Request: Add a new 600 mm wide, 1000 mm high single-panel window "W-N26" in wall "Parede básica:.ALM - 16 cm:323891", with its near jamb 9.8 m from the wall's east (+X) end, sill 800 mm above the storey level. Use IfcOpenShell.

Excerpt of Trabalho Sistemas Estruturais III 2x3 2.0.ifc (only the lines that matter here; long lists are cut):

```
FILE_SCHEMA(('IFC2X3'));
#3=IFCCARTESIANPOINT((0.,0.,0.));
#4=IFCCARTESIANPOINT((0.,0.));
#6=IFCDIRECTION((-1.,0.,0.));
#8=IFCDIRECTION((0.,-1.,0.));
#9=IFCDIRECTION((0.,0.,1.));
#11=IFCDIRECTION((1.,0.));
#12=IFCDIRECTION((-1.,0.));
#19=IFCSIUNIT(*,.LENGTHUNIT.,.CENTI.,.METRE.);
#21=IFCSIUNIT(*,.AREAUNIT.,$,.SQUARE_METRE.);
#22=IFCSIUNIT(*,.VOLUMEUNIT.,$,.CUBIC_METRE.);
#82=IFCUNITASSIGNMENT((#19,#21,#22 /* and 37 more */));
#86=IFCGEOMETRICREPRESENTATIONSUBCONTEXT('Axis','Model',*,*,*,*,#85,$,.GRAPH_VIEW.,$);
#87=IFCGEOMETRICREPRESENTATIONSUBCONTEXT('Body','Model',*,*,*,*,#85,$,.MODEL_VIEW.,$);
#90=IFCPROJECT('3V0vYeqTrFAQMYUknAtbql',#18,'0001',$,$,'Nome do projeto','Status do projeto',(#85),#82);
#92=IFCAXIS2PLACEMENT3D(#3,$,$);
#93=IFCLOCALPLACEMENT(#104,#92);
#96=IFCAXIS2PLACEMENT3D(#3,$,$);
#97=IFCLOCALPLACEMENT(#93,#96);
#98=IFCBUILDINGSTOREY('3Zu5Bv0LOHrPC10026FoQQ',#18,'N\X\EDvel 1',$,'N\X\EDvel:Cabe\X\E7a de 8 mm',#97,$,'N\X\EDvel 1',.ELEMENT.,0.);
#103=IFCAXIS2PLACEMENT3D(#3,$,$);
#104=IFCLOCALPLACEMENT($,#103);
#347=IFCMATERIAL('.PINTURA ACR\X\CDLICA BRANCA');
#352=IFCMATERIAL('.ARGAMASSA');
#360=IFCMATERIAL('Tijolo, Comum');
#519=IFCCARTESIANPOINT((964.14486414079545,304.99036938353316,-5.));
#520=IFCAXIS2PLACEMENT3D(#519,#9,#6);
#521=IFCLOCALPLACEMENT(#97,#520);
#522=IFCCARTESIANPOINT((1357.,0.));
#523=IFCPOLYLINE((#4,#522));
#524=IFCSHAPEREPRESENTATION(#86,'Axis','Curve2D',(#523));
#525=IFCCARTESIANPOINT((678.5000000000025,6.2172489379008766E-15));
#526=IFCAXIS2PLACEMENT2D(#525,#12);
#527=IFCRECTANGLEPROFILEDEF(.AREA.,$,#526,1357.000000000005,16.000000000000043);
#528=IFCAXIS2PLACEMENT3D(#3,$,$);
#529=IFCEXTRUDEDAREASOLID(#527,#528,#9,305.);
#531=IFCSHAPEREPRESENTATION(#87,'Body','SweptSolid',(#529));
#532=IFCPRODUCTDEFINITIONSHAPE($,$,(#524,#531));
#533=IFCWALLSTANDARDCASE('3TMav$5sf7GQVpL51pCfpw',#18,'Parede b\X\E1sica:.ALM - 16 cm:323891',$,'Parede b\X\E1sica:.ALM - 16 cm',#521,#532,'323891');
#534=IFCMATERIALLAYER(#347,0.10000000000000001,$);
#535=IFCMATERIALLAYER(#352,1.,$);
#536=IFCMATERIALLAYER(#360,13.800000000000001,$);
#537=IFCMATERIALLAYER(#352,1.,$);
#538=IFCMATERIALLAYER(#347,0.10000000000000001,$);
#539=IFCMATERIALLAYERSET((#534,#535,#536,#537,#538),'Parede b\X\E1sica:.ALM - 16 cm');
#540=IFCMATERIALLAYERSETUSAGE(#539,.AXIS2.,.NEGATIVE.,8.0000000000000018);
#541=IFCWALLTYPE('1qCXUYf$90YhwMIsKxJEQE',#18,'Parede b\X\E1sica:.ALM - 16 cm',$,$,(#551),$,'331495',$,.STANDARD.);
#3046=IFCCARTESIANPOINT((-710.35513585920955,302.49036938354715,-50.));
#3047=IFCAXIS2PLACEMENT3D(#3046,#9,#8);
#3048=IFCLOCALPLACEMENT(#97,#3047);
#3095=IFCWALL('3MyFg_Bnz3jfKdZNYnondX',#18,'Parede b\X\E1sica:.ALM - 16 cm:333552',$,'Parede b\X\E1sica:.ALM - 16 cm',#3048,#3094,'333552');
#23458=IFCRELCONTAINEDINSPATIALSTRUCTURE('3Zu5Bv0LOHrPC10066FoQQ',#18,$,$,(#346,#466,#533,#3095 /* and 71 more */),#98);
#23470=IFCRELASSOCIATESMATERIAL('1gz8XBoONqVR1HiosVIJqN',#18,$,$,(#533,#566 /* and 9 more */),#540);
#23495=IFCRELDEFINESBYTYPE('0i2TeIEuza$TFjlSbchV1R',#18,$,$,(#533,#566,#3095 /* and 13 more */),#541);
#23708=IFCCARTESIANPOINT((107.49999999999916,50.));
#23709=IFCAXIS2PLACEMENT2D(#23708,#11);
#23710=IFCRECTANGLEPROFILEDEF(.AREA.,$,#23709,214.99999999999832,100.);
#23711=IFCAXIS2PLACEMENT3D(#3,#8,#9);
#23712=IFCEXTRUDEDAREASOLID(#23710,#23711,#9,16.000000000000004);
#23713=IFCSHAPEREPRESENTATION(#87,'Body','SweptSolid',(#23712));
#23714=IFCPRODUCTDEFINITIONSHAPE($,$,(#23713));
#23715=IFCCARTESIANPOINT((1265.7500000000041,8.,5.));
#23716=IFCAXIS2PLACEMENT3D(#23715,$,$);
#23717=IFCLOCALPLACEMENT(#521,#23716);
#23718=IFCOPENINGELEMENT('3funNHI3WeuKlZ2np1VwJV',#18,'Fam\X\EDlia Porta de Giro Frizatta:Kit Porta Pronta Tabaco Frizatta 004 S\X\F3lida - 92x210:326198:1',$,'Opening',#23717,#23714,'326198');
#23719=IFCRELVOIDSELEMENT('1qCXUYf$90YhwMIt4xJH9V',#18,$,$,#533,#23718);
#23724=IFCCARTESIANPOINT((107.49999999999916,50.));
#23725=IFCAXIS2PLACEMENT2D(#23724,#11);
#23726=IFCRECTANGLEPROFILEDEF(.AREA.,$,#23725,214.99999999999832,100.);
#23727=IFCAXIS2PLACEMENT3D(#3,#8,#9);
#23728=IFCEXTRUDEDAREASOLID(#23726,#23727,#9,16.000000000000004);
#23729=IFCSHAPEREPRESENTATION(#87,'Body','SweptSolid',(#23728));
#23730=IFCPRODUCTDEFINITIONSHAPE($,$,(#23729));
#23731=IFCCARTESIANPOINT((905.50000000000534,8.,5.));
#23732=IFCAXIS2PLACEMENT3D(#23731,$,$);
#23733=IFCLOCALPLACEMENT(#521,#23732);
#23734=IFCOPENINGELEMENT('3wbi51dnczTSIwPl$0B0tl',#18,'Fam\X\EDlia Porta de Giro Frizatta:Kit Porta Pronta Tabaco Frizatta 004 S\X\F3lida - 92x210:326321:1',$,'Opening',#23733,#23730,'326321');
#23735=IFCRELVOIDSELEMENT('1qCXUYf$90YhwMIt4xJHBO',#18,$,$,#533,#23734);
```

```python
import numpy as np
import ifcopenshell
import ifcopenshell.api.feature
import ifcopenshell.api.geometry
import ifcopenshell.api.root
import ifcopenshell.api.spatial
import ifcopenshell.api.type
import ifcopenshell.geom
import ifcopenshell.util.element
import ifcopenshell.util.placement
import ifcopenshell.util.representation
import ifcopenshell.util.shape
import ifcopenshell.util.unit

model = ifcopenshell.open("Trabalho Sistemas Estruturais III 2x3 2.0.ifc")
unit_scale = ifcopenshell.util.unit.calculate_unit_scale(model)
settings = ifcopenshell.geom.settings()


def volume(element):
    """Net volume in cubic metres, openings subtracted."""
    shape = ifcopenshell.geom.create_shape(settings, element)
    return ifcopenshell.util.shape.get_volume(shape.geometry)


wall = model.by_guid("3TMav$5sf7GQVpL51pCfpw")
storey = ifcopenshell.util.element.get_container(wall, ifc_class="IfcBuildingStorey")
context = ifcopenshell.util.representation.get_context(model, "Model", "Body", "MODEL_VIEW")
before = volume(wall)

width, height, from_end, sill = 0.6, 1, 9.8, 0.8  # metres

# The wall runs along its own X axis, and the end named is its -X end.
wall_shape = ifcopenshell.geom.create_shape(settings, wall)
x, y, z = ifcopenshell.util.shape.get_vertices(wall_shape.geometry).T
start = x.min() + from_end
face, thickness = float(y.min()), float(y.max() - y.min())
wall_matrix = ifcopenshell.util.placement.get_local_placement(wall.ObjectPlacement)
level = ifcopenshell.util.placement.get_local_placement(storey.ObjectPlacement)[2, 3]


def in_wall(x, y):
    """Placement at x, y metres in the wall's axes, at sill height."""
    matrix = wall_matrix.copy()
    matrix[:, 3] = wall_matrix @ np.array([x / unit_scale, y / unit_scale, 0.0, 1.0])
    matrix[2, 3] = level + sill / unit_scale
    return matrix


# Opening: a box that overshoots both wall faces by 50 mm.
opening = ifcopenshell.api.root.create_entity(model, ifc_class="IfcOpeningElement")
box = ifcopenshell.api.geometry.add_wall_representation(
    model, context=context, length=width, height=height, thickness=thickness + 0.1
)
ifcopenshell.api.geometry.assign_representation(model, product=opening, representation=box)
ifcopenshell.api.geometry.edit_object_placement(model, product=opening, matrix=in_wall(start, face - 0.05), is_si=False)
ifcopenshell.api.feature.add_feature(model, feature=opening, element=wall)

window = ifcopenshell.api.root.create_entity(model, ifc_class="IfcWindow", name="W-N26")
window.OverallWidth, window.OverallHeight = width / unit_scale, height / unit_scale
body = ifcopenshell.api.geometry.add_window_representation(
    model,
    context=context,
    overall_width=window.OverallWidth,
    overall_height=window.OverallHeight,
    partition_type="SINGLE_PANEL",
)
ifcopenshell.api.geometry.assign_representation(model, product=window, representation=body)
ifcopenshell.api.spatial.assign_container(model, products=[window], relating_structure=storey)
fills = ifcopenshell.api.feature.add_filling(model, opening=opening, element=window)
fills.OwnerHistory = window.OwnerHistory  # required in IFC2X3

# IFC2X3 keeps the operation on the window style.
style = ifcopenshell.api.root.create_entity(model, ifc_class="IfcWindowStyle", name="W-N26")
style.OperationType, style.ConstructionType = "SINGLE_PANEL", "NOTDEFINED"
style.ParameterTakesPrecedence = style.Sizeable = False
ifcopenshell.api.type.assign_type(model, related_objects=[window], relating_type=style)

# Centre the window in the wall's thickness.
ifcopenshell.api.geometry.edit_object_placement(model, product=window, matrix=in_wall(start, face), is_si=False)
window_shape = ifcopenshell.geom.create_shape(settings, window)
depth = ifcopenshell.util.shape.get_vertices(window_shape.geometry)[:, 1]
offset = face + thickness / 2 - (depth.min() + depth.max()) / 2
ifcopenshell.api.geometry.edit_object_placement(model, product=window, matrix=in_wall(start, offset), is_si=False)

after = volume(wall)

print(f"wall volume {before:.3f} -> {after:.3f} m3")

model.write("Trabalho Sistemas Estruturais III 2x3 2.0_v2.ifc")
```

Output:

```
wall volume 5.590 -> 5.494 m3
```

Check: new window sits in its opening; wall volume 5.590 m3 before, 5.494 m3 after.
